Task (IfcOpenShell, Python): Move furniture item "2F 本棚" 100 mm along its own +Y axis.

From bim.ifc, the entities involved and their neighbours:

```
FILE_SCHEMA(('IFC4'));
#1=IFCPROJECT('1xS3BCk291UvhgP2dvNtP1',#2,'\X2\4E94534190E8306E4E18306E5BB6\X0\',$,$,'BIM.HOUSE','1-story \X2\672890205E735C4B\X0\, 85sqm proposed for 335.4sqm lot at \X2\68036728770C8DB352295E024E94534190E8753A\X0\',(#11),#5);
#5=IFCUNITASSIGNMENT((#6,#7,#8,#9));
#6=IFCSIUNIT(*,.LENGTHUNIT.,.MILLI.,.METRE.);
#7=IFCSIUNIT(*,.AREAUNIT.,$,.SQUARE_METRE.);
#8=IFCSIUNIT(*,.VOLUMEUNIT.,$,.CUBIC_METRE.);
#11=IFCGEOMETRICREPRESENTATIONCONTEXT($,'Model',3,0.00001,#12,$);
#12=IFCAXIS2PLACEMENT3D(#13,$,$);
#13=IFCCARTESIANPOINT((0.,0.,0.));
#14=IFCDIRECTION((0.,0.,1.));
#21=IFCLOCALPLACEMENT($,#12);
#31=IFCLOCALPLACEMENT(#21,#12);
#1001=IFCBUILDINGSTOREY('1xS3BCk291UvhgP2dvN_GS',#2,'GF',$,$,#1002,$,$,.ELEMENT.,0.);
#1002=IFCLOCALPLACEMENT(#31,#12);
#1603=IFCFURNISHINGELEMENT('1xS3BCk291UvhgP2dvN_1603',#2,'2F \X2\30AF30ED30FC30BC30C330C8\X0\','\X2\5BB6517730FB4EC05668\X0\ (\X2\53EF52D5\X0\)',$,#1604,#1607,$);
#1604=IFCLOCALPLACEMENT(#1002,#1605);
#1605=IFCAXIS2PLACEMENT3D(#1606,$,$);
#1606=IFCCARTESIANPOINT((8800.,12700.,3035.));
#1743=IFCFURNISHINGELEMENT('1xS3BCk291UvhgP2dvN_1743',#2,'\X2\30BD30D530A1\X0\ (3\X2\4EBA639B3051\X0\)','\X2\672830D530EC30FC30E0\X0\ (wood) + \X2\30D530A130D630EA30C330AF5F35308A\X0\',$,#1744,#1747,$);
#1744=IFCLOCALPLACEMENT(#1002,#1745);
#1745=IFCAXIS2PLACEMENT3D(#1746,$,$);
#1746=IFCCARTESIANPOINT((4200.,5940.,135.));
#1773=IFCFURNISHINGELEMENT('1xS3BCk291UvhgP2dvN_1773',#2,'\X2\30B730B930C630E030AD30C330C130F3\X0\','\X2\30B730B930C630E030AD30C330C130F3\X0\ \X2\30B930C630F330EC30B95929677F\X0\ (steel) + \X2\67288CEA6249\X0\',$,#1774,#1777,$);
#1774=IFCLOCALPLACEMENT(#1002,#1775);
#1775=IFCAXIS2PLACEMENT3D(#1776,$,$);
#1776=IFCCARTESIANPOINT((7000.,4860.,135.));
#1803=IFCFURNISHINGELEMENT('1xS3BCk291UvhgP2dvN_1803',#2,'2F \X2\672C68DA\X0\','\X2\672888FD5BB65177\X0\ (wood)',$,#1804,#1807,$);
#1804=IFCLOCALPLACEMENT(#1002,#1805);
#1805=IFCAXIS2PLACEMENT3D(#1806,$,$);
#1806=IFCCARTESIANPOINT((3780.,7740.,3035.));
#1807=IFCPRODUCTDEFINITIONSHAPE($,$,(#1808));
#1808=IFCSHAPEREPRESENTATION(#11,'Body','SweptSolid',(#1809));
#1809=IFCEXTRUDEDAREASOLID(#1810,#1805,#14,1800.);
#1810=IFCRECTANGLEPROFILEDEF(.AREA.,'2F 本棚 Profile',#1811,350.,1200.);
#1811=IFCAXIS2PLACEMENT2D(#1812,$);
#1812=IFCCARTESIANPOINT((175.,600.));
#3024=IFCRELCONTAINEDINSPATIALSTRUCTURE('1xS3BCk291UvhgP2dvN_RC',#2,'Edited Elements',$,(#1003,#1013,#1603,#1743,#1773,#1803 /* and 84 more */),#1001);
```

```python
import ifcopenshell
import ifcopenshell.api.geometry
import ifcopenshell.util.placement

model = ifcopenshell.open("bim.ifc")

item = model.by_guid("1xS3BCk291UvhgP2dvN_1803")
matrix = ifcopenshell.util.placement.get_local_placement(item.ObjectPlacement)
matrix[:3, 3] += matrix[:3, 1] * 100.0
ifcopenshell.api.geometry.edit_object_placement(model, product=item, matrix=matrix, is_si=False)

print(ifcopenshell.util.placement.get_local_placement(item.ObjectPlacement).round(3) + 0.0)

model.write("bim_edited.ifc")
```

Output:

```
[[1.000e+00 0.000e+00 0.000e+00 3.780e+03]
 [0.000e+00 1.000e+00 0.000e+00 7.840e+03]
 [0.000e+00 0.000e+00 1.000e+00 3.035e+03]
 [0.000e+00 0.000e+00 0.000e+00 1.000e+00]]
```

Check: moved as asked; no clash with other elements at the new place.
